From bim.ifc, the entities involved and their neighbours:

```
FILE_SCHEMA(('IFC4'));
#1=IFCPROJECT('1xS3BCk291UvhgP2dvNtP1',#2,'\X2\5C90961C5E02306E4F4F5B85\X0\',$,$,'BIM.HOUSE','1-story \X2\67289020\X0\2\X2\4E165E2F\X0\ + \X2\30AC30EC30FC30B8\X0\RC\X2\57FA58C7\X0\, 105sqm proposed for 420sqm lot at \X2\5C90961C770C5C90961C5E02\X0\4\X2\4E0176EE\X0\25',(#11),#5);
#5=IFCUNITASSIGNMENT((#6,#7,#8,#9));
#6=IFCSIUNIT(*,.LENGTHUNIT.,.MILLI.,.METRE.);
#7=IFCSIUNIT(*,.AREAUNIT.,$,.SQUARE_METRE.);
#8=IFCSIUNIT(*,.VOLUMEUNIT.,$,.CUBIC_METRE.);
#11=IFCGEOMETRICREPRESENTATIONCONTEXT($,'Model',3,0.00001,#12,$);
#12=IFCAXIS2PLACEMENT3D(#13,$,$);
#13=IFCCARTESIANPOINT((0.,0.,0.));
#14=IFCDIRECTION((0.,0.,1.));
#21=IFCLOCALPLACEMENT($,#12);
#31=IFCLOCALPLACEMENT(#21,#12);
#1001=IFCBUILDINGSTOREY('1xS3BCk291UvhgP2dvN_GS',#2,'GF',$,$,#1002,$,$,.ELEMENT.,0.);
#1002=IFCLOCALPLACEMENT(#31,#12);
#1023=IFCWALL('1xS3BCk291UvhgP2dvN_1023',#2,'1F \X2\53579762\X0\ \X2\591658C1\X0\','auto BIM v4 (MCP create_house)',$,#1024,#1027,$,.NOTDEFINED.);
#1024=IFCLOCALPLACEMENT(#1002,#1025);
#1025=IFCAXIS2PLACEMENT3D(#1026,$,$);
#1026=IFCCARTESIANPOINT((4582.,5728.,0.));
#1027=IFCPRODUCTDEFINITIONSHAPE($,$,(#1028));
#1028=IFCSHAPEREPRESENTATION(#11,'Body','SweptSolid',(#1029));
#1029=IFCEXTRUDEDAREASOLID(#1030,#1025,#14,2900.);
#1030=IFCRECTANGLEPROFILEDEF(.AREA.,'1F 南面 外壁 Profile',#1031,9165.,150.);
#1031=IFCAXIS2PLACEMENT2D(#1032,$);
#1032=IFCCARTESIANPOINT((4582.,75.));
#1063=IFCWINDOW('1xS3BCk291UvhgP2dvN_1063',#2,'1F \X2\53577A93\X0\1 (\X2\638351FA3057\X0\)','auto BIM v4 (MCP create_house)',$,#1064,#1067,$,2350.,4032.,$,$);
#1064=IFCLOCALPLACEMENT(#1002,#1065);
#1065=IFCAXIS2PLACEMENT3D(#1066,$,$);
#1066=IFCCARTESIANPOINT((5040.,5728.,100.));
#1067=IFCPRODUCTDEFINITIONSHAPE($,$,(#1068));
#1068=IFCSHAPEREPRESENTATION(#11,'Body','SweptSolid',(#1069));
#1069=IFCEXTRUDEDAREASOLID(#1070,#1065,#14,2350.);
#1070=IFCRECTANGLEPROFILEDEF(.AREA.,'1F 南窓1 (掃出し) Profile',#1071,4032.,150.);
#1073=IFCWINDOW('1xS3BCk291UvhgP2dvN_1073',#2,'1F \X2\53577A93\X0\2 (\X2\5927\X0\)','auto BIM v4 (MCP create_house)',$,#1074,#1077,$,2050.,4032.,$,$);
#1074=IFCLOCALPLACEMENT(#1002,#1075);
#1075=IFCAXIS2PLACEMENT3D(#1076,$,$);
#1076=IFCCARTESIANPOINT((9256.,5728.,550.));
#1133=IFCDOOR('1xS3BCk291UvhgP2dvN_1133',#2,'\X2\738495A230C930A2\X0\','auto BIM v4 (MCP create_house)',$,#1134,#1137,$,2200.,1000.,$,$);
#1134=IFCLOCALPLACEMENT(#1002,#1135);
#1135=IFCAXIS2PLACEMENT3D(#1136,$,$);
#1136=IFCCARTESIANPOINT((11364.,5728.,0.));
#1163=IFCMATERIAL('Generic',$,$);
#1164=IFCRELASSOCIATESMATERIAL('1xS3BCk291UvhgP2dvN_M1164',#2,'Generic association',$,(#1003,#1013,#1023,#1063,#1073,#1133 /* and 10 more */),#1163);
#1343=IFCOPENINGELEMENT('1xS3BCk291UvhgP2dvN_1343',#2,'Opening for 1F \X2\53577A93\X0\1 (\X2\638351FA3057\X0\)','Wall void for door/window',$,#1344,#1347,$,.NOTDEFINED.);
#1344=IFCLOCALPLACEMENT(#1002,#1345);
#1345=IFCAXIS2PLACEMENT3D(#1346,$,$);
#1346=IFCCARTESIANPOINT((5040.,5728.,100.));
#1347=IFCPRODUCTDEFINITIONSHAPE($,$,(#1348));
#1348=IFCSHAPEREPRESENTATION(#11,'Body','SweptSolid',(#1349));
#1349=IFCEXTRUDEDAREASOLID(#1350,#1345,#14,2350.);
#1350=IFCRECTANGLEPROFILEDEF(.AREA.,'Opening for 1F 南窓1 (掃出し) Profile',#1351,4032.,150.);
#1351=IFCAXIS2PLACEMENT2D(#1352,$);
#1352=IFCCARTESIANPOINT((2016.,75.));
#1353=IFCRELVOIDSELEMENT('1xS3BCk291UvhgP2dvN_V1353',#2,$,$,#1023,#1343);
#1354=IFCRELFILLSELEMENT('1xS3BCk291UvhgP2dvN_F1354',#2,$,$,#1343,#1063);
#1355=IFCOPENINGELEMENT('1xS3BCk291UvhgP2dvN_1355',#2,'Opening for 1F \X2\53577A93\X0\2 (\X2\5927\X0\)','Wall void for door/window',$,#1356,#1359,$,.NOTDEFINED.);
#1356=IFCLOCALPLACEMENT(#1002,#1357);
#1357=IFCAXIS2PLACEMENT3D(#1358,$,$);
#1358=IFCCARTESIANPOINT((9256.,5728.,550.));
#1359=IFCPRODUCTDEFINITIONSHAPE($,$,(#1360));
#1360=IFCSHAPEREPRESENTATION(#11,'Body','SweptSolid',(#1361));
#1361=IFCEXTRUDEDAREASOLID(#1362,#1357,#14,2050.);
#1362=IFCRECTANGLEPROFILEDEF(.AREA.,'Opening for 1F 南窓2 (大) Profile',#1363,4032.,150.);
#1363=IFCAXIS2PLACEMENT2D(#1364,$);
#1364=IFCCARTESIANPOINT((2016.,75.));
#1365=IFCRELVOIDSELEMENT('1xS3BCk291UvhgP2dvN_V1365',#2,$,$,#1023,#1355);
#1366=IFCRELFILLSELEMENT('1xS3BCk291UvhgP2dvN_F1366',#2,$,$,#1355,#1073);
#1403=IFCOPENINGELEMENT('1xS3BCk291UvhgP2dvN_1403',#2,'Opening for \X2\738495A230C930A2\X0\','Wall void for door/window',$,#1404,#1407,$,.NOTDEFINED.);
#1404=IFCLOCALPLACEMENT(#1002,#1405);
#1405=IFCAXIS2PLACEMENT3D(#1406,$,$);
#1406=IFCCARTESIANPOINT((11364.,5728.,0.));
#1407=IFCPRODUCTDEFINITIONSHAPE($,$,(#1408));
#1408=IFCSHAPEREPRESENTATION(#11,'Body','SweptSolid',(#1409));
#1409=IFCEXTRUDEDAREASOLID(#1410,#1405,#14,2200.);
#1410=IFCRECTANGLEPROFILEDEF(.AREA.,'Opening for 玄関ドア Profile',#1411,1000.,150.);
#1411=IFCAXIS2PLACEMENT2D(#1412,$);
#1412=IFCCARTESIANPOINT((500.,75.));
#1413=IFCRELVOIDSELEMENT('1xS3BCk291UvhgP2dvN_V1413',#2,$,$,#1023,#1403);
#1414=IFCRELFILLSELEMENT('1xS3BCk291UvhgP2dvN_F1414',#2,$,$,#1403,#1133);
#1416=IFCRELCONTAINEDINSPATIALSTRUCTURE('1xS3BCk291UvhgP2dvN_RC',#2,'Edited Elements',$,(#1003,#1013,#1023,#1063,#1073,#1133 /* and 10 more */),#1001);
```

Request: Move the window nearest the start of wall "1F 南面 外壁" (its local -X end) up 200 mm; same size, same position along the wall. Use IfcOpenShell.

```python
import numpy as np
import ifcopenshell
import ifcopenshell.api.geometry
import ifcopenshell.util.placement
import ifcopenshell.util.unit

model = ifcopenshell.open("bim.ifc")
unit_scale = ifcopenshell.util.unit.calculate_unit_scale(model)

window = model.by_guid("1xS3BCk291UvhgP2dvN_1063")
opening = window.FillsVoids[0].RelatingOpeningElement
dz = 0.2 / unit_scale

shift = np.array([0.0, 0.0, dz])
# The window is not placed relative to its opening, so move both.
for product in (opening, window):
    matrix = ifcopenshell.util.placement.get_local_placement(product.ObjectPlacement)
    matrix[:3, 3] += shift
    ifcopenshell.api.geometry.edit_object_placement(model, product=product, matrix=matrix, is_si=False)

print(f"moved by {dz * unit_scale:+.3f} m")

model.write("bim-out.ifc")
```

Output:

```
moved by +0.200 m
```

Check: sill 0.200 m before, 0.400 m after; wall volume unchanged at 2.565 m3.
